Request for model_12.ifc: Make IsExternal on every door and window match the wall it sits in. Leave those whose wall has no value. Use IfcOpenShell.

First a look at what the model holds.

```python
import ifcopenshell
import ifcopenshell.util.element

model = ifcopenshell.open("model_12.ifc")
print(model.schema)
seen = {}
for e in model.by_type("IfcDoor") + model.by_type("IfcWindow"):
    if not e.FillsVoids:
        continue
    host = e.FillsVoids[0].RelatingOpeningElement.VoidsElements[0].RelatingBuildingElement
    own = ifcopenshell.util.element.get_pset(e, f"Pset_{e.is_a()[3:].removesuffix('StandardCase')}Common", "IsExternal")
    wall = ifcopenshell.util.element.get_pset(host, "Pset_WallCommon", "IsExternal")
    seen[e.is_a(), own, wall] = seen.get((e.is_a(), own, wall), 0) + 1
for (cls, own, wall), count in sorted(seen.items(), key=str):
    print(count, cls, "IsExternal:", own, "| host wall:", wall)
```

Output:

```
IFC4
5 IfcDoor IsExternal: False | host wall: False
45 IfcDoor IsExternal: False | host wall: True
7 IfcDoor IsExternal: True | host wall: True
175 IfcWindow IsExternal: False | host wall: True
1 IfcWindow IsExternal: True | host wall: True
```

```python
import ifcopenshell
import ifcopenshell.api.pset
import ifcopenshell.util.element

model = ifcopenshell.open("model_12.ifc")

count = 0
for ifc_class, pset_name in (("IfcDoor", "Pset_DoorCommon"), ("IfcWindow", "Pset_WindowCommon")):
    for e in model.by_type(ifc_class):
        if not e.FillsVoids:
            continue
        host = e.FillsVoids[0].RelatingOpeningElement.VoidsElements[0].RelatingBuildingElement
        external = ifcopenshell.util.element.get_pset(host, "Pset_WallCommon", "IsExternal")
        if external is None or ifcopenshell.util.element.get_pset(e, pset_name, "IsExternal") == external:
            continue
        pset = ifcopenshell.api.pset.add_pset(model, product=e, name=pset_name)
        ifcopenshell.api.pset.edit_pset(model, pset=pset, properties={"IsExternal": external})
        count += 1

print(count, "updated")

model.write("model_12-out.ifc")
```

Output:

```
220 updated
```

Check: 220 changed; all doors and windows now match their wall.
